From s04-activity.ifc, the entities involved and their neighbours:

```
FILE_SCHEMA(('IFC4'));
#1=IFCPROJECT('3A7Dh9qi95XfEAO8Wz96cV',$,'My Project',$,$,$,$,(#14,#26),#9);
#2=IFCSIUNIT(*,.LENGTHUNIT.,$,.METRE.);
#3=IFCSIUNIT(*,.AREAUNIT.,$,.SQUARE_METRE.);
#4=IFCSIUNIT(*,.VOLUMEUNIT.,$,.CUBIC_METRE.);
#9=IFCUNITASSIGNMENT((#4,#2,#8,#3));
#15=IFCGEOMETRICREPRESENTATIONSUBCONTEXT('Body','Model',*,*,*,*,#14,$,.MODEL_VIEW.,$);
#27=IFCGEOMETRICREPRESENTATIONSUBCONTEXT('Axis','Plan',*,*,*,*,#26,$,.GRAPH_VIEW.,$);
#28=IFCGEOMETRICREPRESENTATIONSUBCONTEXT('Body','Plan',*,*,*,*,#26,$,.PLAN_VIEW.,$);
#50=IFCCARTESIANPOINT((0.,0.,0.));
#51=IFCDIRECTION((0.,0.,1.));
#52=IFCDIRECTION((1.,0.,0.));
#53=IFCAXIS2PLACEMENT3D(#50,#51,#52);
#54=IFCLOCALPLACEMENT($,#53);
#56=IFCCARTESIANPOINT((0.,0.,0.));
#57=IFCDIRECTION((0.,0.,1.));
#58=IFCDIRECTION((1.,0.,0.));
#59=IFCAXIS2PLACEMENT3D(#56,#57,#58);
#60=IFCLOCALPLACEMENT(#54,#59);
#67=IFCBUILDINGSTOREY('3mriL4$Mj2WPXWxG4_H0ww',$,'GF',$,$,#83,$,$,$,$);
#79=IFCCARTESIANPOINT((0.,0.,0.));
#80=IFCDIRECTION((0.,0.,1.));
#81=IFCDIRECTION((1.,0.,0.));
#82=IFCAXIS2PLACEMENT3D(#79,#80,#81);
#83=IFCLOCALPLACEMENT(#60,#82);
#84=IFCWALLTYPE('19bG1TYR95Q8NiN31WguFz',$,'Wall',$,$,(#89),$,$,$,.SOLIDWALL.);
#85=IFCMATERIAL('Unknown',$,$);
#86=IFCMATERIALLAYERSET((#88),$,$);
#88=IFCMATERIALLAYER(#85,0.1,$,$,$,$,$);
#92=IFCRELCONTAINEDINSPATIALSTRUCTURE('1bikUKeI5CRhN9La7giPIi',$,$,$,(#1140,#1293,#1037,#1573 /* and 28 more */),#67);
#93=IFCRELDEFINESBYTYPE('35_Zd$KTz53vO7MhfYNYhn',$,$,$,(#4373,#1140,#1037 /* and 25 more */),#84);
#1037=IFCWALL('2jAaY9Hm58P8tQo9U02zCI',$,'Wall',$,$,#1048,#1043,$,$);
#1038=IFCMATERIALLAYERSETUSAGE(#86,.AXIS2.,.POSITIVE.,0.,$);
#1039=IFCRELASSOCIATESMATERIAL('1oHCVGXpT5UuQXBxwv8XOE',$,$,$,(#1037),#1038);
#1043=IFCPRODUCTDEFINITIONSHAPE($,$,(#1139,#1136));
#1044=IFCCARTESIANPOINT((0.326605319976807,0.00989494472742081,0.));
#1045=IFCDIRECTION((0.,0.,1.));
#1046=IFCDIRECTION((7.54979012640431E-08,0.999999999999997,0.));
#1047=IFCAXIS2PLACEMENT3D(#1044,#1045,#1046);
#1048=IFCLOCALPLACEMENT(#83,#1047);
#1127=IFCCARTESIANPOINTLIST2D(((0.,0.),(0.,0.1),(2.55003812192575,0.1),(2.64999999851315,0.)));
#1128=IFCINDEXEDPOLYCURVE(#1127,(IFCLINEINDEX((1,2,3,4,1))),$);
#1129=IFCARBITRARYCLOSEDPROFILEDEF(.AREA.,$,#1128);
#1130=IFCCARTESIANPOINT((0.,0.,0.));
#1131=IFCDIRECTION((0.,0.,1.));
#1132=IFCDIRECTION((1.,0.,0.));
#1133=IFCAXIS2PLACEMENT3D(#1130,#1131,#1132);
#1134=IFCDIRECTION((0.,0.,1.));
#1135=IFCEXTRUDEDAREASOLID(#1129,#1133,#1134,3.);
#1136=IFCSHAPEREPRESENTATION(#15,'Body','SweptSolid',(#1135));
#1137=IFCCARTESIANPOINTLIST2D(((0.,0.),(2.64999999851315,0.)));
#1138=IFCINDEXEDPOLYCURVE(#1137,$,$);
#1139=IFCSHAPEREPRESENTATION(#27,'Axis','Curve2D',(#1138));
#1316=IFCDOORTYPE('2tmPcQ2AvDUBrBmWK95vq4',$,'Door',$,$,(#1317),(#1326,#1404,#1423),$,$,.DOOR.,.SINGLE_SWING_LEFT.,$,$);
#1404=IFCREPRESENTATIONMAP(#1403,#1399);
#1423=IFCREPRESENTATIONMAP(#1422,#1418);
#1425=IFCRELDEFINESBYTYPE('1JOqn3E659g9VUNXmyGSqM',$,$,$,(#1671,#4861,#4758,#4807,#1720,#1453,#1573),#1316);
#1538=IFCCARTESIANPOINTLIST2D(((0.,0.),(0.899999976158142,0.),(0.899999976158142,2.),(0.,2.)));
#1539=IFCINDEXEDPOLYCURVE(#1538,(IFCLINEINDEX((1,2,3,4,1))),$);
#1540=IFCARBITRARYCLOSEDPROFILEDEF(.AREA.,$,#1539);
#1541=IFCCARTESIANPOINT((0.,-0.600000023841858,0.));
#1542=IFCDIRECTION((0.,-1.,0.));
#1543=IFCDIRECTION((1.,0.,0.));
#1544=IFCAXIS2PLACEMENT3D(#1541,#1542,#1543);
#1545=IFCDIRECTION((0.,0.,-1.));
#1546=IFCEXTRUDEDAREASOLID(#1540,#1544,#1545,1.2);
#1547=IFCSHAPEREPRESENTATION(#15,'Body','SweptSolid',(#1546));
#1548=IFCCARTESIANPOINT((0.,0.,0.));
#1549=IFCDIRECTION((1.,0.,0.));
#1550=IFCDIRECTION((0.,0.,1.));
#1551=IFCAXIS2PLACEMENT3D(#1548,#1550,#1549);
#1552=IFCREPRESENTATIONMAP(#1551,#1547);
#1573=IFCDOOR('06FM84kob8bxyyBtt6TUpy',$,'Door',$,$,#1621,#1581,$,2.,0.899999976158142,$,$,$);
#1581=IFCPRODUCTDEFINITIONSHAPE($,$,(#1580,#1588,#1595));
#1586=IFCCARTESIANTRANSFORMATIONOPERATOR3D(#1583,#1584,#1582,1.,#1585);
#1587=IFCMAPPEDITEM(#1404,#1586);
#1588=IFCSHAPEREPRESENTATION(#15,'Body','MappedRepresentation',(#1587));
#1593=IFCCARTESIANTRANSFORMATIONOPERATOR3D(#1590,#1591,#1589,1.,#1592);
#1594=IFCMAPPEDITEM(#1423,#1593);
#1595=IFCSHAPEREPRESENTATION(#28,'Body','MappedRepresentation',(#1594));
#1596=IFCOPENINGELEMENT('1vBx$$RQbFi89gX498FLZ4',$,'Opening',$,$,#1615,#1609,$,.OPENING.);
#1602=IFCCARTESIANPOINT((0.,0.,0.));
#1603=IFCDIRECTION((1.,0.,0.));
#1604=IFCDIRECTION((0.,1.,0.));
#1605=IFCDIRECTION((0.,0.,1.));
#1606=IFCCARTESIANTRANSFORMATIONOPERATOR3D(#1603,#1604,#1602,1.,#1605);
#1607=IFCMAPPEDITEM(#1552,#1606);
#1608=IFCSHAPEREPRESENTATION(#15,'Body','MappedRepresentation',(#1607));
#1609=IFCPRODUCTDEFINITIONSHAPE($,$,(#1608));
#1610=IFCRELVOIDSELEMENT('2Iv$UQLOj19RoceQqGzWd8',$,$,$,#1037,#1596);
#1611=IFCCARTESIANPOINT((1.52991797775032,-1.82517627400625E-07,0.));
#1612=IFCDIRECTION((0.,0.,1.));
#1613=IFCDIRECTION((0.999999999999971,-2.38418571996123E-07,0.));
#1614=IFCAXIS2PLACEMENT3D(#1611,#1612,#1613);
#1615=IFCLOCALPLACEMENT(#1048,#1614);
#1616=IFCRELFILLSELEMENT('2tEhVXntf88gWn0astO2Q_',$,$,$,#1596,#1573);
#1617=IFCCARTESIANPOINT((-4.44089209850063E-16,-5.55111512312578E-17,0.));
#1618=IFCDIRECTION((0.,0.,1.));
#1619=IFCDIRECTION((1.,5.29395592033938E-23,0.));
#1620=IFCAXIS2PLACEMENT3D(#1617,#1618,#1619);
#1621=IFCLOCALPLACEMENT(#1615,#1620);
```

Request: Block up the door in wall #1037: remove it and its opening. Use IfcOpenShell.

```python
import ifcopenshell
import ifcopenshell.api.feature
import ifcopenshell.api.root
import ifcopenshell.geom
import ifcopenshell.util.shape

model = ifcopenshell.open("s04-activity.ifc")
settings = ifcopenshell.geom.settings()


def volume(element):
    """Net volume in cubic metres, openings subtracted."""
    shape = ifcopenshell.geom.create_shape(settings, element)
    return ifcopenshell.util.shape.get_volume(shape.geometry)


door = model.by_id(1573)
opening = door.FillsVoids[0].RelatingOpeningElement
wall = opening.VoidsElements[0].RelatingBuildingElement
before = volume(wall)

ifcopenshell.api.root.remove_product(model, product=door)
ifcopenshell.api.feature.remove_feature(model, feature=opening)

after = volume(wall)

print(f"wall volume {before:.3f} -> {after:.3f} m3")

model.write("s04-activity_rev.ifc")
```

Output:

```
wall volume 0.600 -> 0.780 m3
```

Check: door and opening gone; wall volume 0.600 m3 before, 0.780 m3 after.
